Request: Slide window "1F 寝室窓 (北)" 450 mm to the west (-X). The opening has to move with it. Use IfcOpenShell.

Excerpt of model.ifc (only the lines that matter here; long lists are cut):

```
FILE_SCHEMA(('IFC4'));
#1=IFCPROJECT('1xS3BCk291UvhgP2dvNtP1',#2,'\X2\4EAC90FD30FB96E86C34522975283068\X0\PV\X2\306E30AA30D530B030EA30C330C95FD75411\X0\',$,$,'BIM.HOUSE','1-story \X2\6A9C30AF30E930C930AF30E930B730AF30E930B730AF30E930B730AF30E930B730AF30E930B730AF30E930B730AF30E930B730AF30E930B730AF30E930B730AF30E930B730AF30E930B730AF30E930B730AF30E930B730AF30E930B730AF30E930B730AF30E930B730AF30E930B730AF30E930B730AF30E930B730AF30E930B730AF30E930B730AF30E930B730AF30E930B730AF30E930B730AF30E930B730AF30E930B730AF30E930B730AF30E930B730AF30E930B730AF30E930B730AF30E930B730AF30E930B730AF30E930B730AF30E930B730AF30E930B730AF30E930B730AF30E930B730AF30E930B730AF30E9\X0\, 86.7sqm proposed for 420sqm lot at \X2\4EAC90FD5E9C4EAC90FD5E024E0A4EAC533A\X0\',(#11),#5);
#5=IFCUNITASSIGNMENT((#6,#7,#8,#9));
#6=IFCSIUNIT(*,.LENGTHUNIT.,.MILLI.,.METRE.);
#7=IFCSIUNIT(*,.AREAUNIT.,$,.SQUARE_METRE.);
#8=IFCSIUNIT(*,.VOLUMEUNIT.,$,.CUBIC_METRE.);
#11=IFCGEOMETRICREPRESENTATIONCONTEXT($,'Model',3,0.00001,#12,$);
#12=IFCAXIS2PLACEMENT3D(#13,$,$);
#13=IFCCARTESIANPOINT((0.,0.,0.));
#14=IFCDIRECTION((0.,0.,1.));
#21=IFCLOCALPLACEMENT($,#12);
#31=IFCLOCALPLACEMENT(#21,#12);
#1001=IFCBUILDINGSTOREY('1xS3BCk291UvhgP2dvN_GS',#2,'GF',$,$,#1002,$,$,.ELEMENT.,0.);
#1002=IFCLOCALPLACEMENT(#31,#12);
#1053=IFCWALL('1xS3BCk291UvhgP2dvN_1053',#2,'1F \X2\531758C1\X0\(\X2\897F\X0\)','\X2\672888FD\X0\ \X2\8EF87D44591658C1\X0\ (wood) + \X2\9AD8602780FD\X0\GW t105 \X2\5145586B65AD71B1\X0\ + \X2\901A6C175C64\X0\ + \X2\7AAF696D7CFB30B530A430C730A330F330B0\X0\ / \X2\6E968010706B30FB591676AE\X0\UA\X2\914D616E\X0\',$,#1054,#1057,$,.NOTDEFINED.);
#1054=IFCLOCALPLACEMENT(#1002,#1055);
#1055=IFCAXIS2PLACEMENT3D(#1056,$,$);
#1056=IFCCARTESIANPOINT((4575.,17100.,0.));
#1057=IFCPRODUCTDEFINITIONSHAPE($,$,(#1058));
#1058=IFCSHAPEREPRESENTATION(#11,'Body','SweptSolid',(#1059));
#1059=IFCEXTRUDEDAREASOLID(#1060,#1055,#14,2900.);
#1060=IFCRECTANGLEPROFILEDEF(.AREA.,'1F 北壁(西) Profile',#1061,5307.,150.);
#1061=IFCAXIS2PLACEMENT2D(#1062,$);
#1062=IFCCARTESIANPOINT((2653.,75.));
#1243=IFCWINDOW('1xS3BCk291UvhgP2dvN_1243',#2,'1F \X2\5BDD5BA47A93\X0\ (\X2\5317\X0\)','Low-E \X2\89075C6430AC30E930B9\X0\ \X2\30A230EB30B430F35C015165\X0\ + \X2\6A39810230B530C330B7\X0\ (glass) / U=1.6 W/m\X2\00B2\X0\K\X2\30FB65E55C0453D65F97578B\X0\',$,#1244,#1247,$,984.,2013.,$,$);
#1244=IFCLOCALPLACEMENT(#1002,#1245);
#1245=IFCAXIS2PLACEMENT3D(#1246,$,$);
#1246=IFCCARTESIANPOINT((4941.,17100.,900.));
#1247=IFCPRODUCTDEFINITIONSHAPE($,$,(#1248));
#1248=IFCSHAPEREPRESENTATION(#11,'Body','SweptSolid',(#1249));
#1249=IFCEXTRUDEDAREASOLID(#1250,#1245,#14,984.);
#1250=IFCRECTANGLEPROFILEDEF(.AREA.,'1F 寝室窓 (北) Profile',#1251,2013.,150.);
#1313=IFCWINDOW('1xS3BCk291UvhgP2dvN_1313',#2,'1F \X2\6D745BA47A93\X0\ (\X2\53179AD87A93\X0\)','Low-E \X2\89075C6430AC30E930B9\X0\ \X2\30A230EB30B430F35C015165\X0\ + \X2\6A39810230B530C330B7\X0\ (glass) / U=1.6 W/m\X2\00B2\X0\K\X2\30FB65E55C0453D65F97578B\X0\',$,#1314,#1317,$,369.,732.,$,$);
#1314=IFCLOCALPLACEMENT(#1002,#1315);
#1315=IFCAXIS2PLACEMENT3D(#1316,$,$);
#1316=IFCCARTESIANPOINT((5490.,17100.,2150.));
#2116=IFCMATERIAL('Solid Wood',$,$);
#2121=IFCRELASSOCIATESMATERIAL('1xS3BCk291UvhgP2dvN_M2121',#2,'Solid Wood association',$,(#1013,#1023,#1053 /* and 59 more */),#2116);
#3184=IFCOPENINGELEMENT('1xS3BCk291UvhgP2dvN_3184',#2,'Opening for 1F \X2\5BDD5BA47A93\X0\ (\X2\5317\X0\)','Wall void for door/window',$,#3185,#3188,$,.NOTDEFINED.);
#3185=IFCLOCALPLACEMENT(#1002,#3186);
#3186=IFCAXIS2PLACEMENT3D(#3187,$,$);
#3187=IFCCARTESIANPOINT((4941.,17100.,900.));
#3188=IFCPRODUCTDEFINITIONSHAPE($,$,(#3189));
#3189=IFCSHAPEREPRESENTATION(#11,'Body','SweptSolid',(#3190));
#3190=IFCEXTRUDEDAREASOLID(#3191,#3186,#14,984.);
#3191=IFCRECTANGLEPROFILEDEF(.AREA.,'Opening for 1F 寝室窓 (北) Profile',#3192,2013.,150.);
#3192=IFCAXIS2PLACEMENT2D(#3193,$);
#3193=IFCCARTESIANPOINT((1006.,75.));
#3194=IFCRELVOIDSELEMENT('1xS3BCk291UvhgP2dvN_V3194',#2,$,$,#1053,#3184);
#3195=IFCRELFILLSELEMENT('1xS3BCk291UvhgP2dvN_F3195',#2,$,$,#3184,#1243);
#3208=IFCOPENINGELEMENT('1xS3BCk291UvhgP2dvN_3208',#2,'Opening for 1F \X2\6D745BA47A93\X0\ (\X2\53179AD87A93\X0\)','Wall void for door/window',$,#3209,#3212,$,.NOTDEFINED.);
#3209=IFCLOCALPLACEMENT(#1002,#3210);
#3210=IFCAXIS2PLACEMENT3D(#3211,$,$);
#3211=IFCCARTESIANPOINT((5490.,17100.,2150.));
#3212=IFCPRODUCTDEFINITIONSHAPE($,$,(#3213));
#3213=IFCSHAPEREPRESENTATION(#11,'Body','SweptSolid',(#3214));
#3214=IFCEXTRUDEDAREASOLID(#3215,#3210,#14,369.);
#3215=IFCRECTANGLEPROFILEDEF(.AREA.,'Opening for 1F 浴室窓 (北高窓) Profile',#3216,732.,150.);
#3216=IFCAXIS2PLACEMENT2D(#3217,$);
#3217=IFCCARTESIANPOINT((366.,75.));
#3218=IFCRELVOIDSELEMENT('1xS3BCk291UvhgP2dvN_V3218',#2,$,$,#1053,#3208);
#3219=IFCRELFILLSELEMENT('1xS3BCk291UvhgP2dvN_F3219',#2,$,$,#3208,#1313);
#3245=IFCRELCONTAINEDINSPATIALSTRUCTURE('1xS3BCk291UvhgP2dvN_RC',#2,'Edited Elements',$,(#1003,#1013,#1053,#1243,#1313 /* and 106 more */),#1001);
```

```python
import ifcopenshell
import ifcopenshell.api.geometry
import ifcopenshell.util.placement

model = ifcopenshell.open("model.ifc")

window = model.by_guid("1xS3BCk291UvhgP2dvN_1243")
opening = window.FillsVoids[0].RelatingOpeningElement
wall = opening.VoidsElements[0].RelatingBuildingElement

wall_matrix = ifcopenshell.util.placement.get_local_placement(wall.ObjectPlacement)
shift = wall_matrix[:3, 0] * -450.0
before = ifcopenshell.util.placement.get_local_placement(window.ObjectPlacement)[:3, 3].copy()

# The window is not placed relative to its opening, so move both.
for product in (opening, window):
    matrix = ifcopenshell.util.placement.get_local_placement(product.ObjectPlacement)
    matrix[:3, 3] += shift
    ifcopenshell.api.geometry.edit_object_placement(model, product=product, matrix=matrix, is_si=False)

after = ifcopenshell.util.placement.get_local_placement(window.ObjectPlacement)[:3, 3]
print("window moved by", (after - before).round(3) + 0.0)

model.write("model_v2.ifc")
```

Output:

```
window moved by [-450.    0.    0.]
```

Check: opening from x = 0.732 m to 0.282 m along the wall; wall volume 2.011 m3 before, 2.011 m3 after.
